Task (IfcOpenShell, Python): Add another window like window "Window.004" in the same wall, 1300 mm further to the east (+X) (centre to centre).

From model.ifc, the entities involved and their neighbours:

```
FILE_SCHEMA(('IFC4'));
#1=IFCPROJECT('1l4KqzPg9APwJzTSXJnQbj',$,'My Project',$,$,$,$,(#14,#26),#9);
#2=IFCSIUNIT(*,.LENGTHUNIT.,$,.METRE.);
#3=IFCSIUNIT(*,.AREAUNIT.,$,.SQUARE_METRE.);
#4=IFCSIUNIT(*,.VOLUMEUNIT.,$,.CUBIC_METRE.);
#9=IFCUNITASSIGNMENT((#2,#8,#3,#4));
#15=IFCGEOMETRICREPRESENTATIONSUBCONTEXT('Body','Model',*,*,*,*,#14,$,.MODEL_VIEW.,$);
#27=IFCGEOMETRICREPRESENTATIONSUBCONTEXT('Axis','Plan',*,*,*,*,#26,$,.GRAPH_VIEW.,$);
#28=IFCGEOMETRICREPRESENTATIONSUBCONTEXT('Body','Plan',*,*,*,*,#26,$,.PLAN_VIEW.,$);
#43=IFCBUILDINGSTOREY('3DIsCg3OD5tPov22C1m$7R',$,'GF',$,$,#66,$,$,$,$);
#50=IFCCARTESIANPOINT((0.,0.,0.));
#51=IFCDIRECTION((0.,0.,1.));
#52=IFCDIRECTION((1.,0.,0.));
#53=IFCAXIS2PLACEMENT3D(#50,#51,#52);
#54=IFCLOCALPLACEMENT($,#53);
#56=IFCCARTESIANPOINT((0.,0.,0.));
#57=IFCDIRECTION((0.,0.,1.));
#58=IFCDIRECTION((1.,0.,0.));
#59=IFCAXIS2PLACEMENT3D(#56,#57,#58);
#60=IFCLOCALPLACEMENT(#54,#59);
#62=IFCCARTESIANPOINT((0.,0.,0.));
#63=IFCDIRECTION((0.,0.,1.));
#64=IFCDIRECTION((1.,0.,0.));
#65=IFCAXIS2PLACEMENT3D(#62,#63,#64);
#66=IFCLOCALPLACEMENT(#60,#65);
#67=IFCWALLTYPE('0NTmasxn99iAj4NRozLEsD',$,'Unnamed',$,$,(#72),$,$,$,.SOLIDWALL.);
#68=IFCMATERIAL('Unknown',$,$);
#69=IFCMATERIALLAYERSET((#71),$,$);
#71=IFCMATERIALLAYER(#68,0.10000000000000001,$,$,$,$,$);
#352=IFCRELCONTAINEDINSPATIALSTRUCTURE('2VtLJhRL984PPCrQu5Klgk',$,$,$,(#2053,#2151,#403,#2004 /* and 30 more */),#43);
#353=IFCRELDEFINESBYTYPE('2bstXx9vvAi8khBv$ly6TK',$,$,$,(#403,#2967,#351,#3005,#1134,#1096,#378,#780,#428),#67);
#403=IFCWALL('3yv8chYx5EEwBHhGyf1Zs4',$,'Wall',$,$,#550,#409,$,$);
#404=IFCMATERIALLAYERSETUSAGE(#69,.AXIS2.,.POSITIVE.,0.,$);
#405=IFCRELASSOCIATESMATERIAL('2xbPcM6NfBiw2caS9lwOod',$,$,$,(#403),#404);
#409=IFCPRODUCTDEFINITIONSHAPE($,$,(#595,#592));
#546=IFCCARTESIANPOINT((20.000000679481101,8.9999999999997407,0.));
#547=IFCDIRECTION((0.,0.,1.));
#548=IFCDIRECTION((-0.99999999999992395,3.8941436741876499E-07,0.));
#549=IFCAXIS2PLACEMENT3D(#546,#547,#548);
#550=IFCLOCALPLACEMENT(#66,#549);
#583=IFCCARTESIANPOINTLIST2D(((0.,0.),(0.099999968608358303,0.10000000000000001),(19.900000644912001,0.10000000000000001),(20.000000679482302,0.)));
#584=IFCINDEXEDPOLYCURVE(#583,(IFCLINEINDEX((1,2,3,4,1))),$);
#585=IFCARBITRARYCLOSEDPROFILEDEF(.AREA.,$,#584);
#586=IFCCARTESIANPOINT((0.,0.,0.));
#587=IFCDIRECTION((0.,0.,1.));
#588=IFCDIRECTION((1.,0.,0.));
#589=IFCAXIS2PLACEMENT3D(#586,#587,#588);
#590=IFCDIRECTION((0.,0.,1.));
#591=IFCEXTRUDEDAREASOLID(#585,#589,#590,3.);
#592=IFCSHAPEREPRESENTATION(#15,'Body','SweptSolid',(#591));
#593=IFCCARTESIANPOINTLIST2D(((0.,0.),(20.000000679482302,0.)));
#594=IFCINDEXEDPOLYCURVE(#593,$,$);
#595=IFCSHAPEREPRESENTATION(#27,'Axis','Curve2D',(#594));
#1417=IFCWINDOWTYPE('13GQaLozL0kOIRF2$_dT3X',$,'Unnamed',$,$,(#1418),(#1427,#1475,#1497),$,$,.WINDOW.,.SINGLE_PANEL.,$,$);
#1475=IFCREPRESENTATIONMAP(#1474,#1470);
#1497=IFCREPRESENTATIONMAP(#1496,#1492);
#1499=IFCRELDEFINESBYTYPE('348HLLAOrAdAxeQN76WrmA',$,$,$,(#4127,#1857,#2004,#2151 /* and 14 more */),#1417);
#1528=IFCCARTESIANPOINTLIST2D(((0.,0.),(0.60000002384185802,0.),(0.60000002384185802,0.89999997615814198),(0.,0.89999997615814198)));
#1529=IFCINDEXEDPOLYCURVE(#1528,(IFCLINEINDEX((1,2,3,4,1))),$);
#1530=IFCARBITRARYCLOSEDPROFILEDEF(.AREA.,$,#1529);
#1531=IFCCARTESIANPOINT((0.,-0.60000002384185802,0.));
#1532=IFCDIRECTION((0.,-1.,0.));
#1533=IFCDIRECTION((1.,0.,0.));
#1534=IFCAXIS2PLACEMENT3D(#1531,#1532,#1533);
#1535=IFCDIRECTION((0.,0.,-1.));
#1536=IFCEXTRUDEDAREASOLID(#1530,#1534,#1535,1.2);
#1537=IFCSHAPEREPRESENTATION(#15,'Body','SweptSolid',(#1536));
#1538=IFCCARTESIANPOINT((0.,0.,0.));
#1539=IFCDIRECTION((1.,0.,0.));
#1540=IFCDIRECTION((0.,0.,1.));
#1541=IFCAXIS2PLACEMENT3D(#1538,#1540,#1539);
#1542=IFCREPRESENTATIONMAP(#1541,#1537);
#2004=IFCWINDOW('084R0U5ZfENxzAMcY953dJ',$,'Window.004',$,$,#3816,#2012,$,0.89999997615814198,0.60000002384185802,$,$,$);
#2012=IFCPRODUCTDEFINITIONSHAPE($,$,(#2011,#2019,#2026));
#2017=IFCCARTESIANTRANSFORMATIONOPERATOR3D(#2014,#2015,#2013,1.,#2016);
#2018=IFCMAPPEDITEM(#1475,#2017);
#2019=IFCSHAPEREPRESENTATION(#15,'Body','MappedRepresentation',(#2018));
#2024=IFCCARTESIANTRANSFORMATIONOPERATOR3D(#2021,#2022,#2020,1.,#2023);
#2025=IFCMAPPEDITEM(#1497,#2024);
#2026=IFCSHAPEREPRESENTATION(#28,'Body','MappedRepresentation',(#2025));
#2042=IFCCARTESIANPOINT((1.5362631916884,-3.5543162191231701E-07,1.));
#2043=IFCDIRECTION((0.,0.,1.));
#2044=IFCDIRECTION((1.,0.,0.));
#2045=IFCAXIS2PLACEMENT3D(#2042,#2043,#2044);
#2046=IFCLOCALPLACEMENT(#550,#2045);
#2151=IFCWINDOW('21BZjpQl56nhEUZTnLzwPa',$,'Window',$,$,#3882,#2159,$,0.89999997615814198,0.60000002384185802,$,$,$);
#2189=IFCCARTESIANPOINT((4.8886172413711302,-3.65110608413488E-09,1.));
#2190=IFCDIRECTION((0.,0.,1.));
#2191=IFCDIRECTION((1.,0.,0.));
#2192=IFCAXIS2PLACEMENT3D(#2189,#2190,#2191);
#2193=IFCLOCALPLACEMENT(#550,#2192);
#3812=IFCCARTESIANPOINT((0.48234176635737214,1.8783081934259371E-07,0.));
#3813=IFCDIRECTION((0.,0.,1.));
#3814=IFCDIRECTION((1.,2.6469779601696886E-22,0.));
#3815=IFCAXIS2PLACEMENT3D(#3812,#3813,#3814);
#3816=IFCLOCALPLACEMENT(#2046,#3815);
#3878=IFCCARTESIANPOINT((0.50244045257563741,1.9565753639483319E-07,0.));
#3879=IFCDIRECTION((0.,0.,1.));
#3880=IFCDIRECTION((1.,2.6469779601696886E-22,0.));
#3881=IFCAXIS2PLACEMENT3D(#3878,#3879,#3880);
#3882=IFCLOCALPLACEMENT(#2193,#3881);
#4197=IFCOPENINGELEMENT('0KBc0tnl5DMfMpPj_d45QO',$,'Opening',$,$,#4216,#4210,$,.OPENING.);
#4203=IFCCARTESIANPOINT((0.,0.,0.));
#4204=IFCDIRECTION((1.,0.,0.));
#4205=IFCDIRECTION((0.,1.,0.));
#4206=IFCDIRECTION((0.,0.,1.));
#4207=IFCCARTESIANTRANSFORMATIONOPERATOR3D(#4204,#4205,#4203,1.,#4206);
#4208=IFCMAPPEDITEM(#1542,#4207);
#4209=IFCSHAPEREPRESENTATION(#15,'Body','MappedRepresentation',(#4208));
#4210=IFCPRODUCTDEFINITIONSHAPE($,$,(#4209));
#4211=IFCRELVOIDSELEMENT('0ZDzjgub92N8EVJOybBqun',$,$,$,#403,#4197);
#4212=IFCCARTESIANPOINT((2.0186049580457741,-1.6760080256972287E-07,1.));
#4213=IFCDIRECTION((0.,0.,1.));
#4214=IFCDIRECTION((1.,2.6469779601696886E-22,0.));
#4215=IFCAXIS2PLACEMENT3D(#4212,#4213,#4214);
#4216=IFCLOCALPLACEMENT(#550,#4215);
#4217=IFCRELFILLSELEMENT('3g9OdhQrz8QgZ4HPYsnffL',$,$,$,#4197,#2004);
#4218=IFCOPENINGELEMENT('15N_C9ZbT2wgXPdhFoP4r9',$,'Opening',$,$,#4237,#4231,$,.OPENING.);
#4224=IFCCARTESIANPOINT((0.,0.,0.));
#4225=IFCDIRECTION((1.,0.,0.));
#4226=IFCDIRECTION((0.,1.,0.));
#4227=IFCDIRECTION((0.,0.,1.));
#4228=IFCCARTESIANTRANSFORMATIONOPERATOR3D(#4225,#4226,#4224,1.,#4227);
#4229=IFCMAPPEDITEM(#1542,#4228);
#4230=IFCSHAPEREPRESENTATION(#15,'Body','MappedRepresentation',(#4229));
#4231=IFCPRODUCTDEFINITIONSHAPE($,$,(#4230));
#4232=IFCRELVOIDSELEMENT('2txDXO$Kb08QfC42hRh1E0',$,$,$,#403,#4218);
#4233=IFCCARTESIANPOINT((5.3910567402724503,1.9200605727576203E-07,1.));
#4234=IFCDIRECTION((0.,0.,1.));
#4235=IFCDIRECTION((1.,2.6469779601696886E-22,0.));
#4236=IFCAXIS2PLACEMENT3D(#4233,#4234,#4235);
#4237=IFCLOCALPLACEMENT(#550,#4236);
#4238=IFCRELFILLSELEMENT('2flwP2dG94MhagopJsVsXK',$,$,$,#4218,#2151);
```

```python
import ifcopenshell
import ifcopenshell.api.feature
import ifcopenshell.api.geometry
import ifcopenshell.api.root
import ifcopenshell.geom
import ifcopenshell.util.element
import ifcopenshell.util.placement
import ifcopenshell.util.shape
import ifcopenshell.util.unit

model = ifcopenshell.open("model.ifc")
unit_scale = ifcopenshell.util.unit.calculate_unit_scale(model)
settings = ifcopenshell.geom.settings()


def volume(element):
    """Net volume in cubic metres, openings subtracted."""
    shape = ifcopenshell.geom.create_shape(settings, element)
    return ifcopenshell.util.shape.get_volume(shape.geometry)


window = model.by_guid("084R0U5ZfENxzAMcY953dJ")
opening = window.FillsVoids[0].RelatingOpeningElement
wall = opening.VoidsElements[0].RelatingBuildingElement
before = volume(wall)
shift = ifcopenshell.util.placement.get_local_placement(wall.ObjectPlacement)[:3, 0] * -1.3 / unit_scale

# copy_class copies the void relationship, type, container and properties, but no geometry.
new_opening = ifcopenshell.api.root.copy_class(model, product=opening)
new_opening.Representation = ifcopenshell.util.element.copy_deep(
    model, opening.Representation, exclude=["IfcGeometricRepresentationContext", "IfcRepresentationMap"]
)
new_window = ifcopenshell.api.root.copy_class(model, product=window)
new_window.Representation = ifcopenshell.util.element.copy_deep(
    model, window.Representation, exclude=["IfcGeometricRepresentationContext", "IfcRepresentationMap"]
)
ifcopenshell.api.feature.add_filling(model, opening=new_opening, element=new_window)

for old, new in ((opening, new_opening), (window, new_window)):
    matrix = ifcopenshell.util.placement.get_local_placement(old.ObjectPlacement)
    matrix[:3, 3] += shift
    ifcopenshell.api.geometry.edit_object_placement(model, product=new, matrix=matrix, is_si=False)

after = volume(wall)

print(f"wall volume {before:.3f} -> {after:.3f} m3")

model.write("model-out.ifc")
```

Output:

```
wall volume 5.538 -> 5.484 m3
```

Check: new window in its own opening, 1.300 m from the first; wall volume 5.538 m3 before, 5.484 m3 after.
